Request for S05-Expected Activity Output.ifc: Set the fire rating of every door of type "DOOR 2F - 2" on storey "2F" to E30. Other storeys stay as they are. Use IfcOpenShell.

First a look at what the model holds.

```python
import ifcopenshell
import ifcopenshell.util.element

model = ifcopenshell.open("S05-Expected Activity Output.ifc")
print(model.schema)
storey = next(s for s in model.by_type("IfcBuildingStorey") if s.Name == "2F")
doors = [e for e in ifcopenshell.util.element.get_decomposition(storey) if e.is_a("IfcDoor")]
seen = {}
for e in doors:
    element_type = ifcopenshell.util.element.get_type(e)
    key = (element_type.Name if element_type != e and element_type else None, ifcopenshell.util.element.get_pset(e, "Pset_DoorCommon", "FireRating"))
    seen[key] = seen.get(key, 0) + 1
for (name, value), count in sorted(seen.items(), key=str):
    print(count, "x", name, "|", value)
```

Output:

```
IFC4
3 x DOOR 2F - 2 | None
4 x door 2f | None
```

```python
import ifcopenshell
import ifcopenshell.api.pset
import ifcopenshell.util.element

model = ifcopenshell.open("S05-Expected Activity Output.ifc")

storey = next(s for s in model.by_type("IfcBuildingStorey") if s.Name == "2F")
doors = [e for e in ifcopenshell.util.element.get_decomposition(storey) if e.is_a("IfcDoor")]

count = 0
for e in doors:
    element_type = ifcopenshell.util.element.get_type(e)
    if element_type in (None, e) or element_type.Name != "DOOR 2F - 2":
        continue
    # add_pset returns the element's existing set when there is one.
    pset = ifcopenshell.api.pset.add_pset(model, product=e, name="Pset_DoorCommon")
    ifcopenshell.api.pset.edit_pset(model, pset=pset, properties={"FireRating": "E30"})
    count += 1

print(count, "doors updated")

model.write("S05-Expected Activity Output_v2.ifc")
```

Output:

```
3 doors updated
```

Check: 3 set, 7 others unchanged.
